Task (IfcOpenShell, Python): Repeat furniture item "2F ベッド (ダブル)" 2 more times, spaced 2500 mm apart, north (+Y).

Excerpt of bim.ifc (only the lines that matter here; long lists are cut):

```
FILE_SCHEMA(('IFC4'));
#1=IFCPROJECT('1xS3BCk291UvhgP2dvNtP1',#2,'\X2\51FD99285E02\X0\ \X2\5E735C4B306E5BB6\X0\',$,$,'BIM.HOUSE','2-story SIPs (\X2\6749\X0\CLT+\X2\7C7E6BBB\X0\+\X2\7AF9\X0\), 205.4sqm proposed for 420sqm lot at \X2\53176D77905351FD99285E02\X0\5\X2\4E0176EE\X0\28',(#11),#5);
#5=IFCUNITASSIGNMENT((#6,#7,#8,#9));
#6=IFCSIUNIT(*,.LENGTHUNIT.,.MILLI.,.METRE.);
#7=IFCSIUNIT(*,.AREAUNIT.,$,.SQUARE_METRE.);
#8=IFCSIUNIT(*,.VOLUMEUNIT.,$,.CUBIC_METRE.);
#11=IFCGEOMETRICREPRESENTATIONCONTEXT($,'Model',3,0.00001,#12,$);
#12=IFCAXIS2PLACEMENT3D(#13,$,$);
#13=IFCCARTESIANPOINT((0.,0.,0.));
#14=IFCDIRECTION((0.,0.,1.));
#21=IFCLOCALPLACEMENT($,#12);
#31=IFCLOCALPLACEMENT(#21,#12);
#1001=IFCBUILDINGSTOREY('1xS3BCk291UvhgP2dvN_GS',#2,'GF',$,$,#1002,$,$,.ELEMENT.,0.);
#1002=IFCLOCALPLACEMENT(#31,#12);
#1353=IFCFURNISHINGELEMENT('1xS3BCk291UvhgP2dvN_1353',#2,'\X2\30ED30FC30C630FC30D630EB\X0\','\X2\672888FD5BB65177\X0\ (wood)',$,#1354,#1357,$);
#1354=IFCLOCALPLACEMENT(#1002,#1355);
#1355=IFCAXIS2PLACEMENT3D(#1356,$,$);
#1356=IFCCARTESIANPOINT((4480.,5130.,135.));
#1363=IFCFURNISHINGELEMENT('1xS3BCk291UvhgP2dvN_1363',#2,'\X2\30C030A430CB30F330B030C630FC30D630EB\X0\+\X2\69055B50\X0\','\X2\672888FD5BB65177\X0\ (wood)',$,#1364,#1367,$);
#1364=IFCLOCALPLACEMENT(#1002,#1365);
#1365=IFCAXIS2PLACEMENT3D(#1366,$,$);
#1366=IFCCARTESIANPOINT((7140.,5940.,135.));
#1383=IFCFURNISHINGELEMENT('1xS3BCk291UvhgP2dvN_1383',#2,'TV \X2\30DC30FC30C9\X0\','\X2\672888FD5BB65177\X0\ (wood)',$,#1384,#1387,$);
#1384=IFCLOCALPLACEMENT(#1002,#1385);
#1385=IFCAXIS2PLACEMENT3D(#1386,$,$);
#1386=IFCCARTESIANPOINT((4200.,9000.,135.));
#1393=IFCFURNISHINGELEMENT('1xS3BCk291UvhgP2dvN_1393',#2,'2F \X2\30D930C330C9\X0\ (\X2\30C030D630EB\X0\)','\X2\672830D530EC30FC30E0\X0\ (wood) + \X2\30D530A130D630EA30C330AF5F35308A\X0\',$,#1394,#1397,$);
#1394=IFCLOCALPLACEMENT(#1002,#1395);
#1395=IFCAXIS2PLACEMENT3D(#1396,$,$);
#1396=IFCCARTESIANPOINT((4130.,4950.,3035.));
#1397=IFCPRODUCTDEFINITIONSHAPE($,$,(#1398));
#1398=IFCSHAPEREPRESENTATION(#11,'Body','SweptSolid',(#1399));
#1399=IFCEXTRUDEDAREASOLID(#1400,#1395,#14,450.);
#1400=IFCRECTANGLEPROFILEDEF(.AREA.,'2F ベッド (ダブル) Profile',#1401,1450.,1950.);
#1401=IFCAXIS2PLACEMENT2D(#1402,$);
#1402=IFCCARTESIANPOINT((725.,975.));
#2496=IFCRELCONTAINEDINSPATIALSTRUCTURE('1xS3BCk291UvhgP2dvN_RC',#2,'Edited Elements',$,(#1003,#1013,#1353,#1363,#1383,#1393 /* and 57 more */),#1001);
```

```python
import numpy as np
import ifcopenshell
import ifcopenshell.api.geometry
import ifcopenshell.api.root
import ifcopenshell.util.element
import ifcopenshell.util.placement

model = ifcopenshell.open("bim.ifc")


def reuse_history(source, copy):
    """copy_class also copies each property set's owner history, people and application; keep the originals."""
    for rel in copy.IsDefinedBy:
        if rel.is_a("IfcRelDefinesByProperties") and (history := rel.RelatingPropertyDefinition.OwnerHistory):
            rel.RelatingPropertyDefinition.OwnerHistory = source.OwnerHistory
            ifcopenshell.util.element.remove_deep2(model, history)


source = model.by_id(1393)
base = ifcopenshell.util.placement.get_local_placement(source.ObjectPlacement)
step = np.array([0.0, 1.0, 0.0]) * 2500.0

for i in range(1, 3):
    copy = ifcopenshell.api.root.copy_class(model, product=source)
    copy.Representation = ifcopenshell.util.element.copy_deep(
        model, source.Representation, exclude=["IfcGeometricRepresentationContext", "IfcRepresentationMap"]
    )
    reuse_history(source, copy)
    matrix = base.copy()
    matrix[:3, 3] += i * step
    print("added at", matrix[:3, 3].round(3) + 0.0)
    ifcopenshell.api.geometry.edit_object_placement(model, product=copy, matrix=matrix, is_si=False)

model.write("bim_edited.ifc")
```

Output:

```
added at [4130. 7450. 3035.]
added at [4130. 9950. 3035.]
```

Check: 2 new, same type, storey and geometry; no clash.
